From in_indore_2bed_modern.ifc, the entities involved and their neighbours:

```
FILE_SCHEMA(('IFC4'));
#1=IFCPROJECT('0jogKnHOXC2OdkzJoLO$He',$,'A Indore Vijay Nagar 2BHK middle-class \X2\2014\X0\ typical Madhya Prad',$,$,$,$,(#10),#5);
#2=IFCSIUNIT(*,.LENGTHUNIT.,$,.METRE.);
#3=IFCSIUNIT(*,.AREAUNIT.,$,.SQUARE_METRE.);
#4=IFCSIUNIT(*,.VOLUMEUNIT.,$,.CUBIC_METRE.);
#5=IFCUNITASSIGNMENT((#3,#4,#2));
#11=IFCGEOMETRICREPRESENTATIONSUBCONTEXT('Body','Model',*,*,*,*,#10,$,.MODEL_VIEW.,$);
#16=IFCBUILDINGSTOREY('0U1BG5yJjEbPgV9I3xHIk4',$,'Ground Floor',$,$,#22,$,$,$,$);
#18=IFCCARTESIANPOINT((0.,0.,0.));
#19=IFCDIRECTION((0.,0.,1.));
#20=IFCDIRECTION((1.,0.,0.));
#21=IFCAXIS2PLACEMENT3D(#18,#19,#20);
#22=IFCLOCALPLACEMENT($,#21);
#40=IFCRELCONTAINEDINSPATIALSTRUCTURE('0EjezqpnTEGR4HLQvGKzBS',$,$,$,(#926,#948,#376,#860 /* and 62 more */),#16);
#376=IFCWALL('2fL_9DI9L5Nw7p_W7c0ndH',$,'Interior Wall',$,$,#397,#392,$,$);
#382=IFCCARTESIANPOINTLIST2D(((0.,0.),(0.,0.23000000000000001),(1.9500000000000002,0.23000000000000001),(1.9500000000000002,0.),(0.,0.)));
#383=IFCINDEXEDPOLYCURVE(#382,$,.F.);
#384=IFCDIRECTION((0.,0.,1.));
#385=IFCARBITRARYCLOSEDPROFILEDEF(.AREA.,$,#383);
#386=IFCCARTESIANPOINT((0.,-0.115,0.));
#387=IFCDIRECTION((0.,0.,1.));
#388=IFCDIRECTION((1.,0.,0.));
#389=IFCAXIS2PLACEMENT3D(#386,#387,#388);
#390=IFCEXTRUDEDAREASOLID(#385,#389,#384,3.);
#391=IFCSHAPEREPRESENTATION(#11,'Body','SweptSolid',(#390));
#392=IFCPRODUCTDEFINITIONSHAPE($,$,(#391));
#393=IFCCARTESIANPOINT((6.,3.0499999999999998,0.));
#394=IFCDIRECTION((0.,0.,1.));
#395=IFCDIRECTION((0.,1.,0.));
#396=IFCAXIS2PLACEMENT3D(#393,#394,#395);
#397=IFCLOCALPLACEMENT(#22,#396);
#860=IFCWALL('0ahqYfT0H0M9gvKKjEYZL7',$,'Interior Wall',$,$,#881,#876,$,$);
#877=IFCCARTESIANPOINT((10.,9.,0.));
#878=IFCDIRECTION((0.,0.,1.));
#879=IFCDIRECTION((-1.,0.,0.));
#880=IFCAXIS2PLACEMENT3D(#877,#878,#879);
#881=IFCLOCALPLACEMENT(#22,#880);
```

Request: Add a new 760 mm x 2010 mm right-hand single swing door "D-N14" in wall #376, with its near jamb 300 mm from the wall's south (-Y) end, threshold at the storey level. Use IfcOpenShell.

```python
import numpy as np
import ifcopenshell
import ifcopenshell.api.feature
import ifcopenshell.api.geometry
import ifcopenshell.api.root
import ifcopenshell.api.spatial
import ifcopenshell.geom
import ifcopenshell.util.element
import ifcopenshell.util.placement
import ifcopenshell.util.representation
import ifcopenshell.util.shape
import ifcopenshell.util.unit

model = ifcopenshell.open("in_indore_2bed_modern.ifc")
unit_scale = ifcopenshell.util.unit.calculate_unit_scale(model)
settings = ifcopenshell.geom.settings()


def volume(element):
    """Net volume in cubic metres, openings subtracted."""
    shape = ifcopenshell.geom.create_shape(settings, element)
    return ifcopenshell.util.shape.get_volume(shape.geometry)


wall = model.by_guid("2fL_9DI9L5Nw7p_W7c0ndH")
storey = ifcopenshell.util.element.get_container(wall, ifc_class="IfcBuildingStorey")
context = ifcopenshell.util.representation.get_context(model, "Model", "Body", "MODEL_VIEW")
before = volume(wall)

width, height, from_end, sill = 0.76, 2.01, 0.3, 0.0  # metres

# The wall runs along its own X axis, and the end named is its -X end.
wall_shape = ifcopenshell.geom.create_shape(settings, wall)
x, y, z = ifcopenshell.util.shape.get_vertices(wall_shape.geometry).T
start = x.min() + from_end
face, thickness = float(y.min()), float(y.max() - y.min())
wall_matrix = ifcopenshell.util.placement.get_local_placement(wall.ObjectPlacement)
level = ifcopenshell.util.placement.get_local_placement(storey.ObjectPlacement)[2, 3]


def in_wall(x, y):
    """Placement at x, y metres in the wall's axes, at sill height."""
    matrix = wall_matrix.copy()
    matrix[:, 3] = wall_matrix @ np.array([x / unit_scale, y / unit_scale, 0.0, 1.0])
    matrix[2, 3] = level + sill / unit_scale
    return matrix


# Opening: a box that overshoots both wall faces by 50 mm.
opening = ifcopenshell.api.root.create_entity(model, ifc_class="IfcOpeningElement", predefined_type="OPENING")
box = ifcopenshell.api.geometry.add_wall_representation(
    model, context=context, length=width, height=height, thickness=thickness + 0.1
)
ifcopenshell.api.geometry.assign_representation(model, product=opening, representation=box)
ifcopenshell.api.geometry.edit_object_placement(model, product=opening, matrix=in_wall(start, face - 0.05), is_si=False)
ifcopenshell.api.feature.add_feature(model, feature=opening, element=wall)

door = ifcopenshell.api.root.create_entity(model, ifc_class="IfcDoor", name="D-N14", predefined_type="DOOR")
door.OverallWidth, door.OverallHeight = width / unit_scale, height / unit_scale
door.OperationType = "SINGLE_SWING_RIGHT"
body = ifcopenshell.api.geometry.add_door_representation(
    model,
    context=context,
    overall_width=door.OverallWidth,
    overall_height=door.OverallHeight,
    operation_type="SINGLE_SWING_RIGHT",
    lining_properties={"LiningDepth": thickness / unit_scale, "ThresholdDepth": thickness / unit_scale},
)
ifcopenshell.api.geometry.assign_representation(model, product=door, representation=body)
ifcopenshell.api.spatial.assign_container(model, products=[door], relating_structure=storey)
ifcopenshell.api.feature.add_filling(model, opening=opening, element=door)

# The lining spans the wall, so the door starts at the wall face.
ifcopenshell.api.geometry.edit_object_placement(model, product=door, matrix=in_wall(start, face), is_si=False)

after = volume(wall)

print(f"wall volume {before:.3f} -> {after:.3f} m3")

model.write("in_indore_2bed_modern_rev.ifc")
```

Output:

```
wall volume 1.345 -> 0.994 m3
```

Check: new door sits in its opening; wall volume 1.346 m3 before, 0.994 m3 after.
